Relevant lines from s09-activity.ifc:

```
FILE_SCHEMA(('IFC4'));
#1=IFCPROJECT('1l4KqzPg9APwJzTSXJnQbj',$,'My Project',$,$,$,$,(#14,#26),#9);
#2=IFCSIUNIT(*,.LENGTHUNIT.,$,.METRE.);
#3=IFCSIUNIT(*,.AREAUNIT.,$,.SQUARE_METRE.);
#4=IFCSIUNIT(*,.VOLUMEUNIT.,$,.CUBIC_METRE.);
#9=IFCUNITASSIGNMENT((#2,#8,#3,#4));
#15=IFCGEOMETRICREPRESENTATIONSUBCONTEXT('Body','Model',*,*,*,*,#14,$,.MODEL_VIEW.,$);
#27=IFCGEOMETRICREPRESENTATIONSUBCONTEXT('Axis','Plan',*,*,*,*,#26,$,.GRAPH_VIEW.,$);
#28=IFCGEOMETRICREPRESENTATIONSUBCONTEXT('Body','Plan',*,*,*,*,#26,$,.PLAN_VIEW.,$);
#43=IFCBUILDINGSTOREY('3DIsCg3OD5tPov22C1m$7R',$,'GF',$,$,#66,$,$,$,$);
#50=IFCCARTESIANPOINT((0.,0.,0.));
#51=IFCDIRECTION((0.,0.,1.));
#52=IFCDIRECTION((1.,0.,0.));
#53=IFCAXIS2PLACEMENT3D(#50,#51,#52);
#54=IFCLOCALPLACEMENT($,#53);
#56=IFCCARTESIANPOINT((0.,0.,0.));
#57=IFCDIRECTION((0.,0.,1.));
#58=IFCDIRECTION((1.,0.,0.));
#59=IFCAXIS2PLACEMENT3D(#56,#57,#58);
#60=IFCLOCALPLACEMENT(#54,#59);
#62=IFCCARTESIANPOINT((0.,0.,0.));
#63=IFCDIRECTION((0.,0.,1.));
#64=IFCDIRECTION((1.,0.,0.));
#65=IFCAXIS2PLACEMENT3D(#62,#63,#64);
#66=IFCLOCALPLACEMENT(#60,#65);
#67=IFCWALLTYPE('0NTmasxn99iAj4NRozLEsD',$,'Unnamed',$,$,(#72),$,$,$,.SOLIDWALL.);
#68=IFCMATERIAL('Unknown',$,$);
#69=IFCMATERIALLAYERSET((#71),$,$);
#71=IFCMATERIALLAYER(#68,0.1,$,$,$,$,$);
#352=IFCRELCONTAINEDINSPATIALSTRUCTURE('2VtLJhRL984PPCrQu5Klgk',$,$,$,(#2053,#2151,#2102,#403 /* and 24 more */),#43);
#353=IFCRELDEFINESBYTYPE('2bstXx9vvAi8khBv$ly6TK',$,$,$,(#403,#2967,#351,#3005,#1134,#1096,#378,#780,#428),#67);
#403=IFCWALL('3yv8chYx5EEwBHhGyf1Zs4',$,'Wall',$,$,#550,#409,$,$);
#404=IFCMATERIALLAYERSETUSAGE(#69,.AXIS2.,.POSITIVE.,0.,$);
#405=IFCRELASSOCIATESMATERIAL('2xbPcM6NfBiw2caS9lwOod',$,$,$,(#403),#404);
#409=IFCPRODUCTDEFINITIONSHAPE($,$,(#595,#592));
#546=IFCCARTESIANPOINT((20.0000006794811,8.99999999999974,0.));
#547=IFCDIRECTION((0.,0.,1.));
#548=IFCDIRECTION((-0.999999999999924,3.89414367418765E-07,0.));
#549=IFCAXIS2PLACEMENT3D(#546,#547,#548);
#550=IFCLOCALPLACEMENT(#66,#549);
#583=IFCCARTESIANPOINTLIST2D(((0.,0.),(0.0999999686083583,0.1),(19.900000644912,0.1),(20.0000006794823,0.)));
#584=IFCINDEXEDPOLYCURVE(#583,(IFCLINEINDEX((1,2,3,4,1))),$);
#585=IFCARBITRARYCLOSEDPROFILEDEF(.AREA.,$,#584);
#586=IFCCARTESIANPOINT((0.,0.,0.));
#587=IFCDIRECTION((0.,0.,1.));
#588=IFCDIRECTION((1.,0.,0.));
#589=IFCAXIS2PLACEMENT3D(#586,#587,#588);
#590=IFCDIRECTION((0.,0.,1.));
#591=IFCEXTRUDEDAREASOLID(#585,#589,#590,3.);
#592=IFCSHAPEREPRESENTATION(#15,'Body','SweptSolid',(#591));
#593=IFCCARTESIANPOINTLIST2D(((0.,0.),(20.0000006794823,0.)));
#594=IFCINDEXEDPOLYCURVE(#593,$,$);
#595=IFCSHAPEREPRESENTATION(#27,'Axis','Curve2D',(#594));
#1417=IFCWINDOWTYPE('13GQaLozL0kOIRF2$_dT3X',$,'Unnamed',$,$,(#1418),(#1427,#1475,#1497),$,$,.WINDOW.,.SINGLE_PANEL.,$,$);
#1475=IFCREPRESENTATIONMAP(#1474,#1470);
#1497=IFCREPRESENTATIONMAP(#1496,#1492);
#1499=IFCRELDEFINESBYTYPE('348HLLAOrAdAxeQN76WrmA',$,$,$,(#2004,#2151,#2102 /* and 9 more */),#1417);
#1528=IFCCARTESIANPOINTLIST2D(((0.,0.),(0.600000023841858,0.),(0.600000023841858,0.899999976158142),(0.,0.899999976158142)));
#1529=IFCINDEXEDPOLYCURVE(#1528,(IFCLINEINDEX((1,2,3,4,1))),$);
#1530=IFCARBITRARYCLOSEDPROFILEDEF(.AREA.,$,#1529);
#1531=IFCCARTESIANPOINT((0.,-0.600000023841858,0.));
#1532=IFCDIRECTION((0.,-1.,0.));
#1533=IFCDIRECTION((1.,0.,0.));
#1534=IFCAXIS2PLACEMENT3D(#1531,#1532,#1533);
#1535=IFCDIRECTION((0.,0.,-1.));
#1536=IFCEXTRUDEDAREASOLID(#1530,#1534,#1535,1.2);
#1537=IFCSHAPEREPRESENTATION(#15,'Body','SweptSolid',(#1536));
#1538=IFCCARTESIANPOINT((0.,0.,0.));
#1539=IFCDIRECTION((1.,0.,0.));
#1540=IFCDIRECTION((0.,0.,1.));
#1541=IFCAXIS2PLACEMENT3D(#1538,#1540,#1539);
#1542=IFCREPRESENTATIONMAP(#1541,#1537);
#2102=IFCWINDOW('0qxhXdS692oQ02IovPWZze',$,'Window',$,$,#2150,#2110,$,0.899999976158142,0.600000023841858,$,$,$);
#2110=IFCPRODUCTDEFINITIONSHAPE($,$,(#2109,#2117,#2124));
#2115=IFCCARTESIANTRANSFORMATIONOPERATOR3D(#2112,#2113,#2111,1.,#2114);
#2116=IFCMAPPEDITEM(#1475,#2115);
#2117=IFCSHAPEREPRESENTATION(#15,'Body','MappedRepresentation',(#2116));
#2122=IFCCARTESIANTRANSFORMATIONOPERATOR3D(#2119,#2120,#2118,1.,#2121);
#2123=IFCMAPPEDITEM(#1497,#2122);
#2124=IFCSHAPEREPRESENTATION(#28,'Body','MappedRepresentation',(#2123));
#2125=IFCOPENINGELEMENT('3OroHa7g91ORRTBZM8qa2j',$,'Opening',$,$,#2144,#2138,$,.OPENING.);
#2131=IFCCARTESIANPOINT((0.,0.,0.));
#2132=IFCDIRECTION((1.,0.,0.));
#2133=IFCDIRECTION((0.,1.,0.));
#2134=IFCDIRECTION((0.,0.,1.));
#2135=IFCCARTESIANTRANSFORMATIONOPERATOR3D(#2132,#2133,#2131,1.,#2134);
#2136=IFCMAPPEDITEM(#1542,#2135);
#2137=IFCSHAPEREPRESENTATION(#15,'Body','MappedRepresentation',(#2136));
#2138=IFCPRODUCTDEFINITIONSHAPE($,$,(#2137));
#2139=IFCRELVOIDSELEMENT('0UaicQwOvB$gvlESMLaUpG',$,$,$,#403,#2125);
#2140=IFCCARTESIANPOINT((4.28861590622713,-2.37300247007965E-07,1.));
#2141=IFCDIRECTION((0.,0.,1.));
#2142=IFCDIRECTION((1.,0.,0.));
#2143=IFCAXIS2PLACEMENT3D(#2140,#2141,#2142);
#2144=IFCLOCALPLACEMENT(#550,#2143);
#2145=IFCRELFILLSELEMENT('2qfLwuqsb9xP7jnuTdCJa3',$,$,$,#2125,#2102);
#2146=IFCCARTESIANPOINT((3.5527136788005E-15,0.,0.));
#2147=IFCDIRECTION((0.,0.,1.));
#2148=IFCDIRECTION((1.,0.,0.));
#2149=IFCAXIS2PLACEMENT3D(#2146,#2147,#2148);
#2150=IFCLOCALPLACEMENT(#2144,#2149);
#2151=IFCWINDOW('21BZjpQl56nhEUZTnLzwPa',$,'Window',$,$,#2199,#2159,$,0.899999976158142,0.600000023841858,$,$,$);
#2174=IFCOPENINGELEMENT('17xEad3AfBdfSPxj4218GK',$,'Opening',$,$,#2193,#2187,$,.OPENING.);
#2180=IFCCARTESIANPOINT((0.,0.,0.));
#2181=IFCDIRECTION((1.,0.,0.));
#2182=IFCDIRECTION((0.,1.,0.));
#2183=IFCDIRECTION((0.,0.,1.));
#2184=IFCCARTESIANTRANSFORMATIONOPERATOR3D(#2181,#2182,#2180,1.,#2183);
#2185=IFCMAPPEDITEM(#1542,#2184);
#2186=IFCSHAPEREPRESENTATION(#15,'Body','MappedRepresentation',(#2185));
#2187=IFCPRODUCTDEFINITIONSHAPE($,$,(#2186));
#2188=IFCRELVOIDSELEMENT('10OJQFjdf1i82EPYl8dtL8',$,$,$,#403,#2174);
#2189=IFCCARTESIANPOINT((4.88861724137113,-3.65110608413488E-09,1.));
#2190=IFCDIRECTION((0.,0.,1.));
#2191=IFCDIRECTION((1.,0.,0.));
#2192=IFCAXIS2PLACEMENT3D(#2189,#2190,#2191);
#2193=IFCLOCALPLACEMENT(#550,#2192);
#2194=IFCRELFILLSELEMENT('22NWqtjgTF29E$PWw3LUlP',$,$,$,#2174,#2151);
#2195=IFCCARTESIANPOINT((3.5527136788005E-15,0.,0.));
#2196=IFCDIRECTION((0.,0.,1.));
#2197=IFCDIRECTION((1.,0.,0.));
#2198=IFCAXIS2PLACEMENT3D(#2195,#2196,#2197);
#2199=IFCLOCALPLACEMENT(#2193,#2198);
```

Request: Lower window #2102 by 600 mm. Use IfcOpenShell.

```python
import numpy as np
import ifcopenshell
import ifcopenshell.api.geometry
import ifcopenshell.util.placement
import ifcopenshell.util.unit

model = ifcopenshell.open("s09-activity.ifc")
unit_scale = ifcopenshell.util.unit.calculate_unit_scale(model)

window = model.by_guid("0qxhXdS692oQ02IovPWZze")
opening = window.FillsVoids[0].RelatingOpeningElement
dz = -0.6

shift = np.array([0.0, 0.0, dz])
# The window is placed relative to its opening, so it follows when the opening moves.
matrix = ifcopenshell.util.placement.get_local_placement(opening.ObjectPlacement)
matrix[:3, 3] += shift
ifcopenshell.api.geometry.edit_object_placement(
    model, product=opening, matrix=matrix, is_si=False, should_transform_children=True
)

print(f"moved by {dz * unit_scale:+.3f} m")

model.write("s09-activity_rev.ifc")
```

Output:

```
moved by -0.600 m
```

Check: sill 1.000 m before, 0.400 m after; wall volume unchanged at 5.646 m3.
